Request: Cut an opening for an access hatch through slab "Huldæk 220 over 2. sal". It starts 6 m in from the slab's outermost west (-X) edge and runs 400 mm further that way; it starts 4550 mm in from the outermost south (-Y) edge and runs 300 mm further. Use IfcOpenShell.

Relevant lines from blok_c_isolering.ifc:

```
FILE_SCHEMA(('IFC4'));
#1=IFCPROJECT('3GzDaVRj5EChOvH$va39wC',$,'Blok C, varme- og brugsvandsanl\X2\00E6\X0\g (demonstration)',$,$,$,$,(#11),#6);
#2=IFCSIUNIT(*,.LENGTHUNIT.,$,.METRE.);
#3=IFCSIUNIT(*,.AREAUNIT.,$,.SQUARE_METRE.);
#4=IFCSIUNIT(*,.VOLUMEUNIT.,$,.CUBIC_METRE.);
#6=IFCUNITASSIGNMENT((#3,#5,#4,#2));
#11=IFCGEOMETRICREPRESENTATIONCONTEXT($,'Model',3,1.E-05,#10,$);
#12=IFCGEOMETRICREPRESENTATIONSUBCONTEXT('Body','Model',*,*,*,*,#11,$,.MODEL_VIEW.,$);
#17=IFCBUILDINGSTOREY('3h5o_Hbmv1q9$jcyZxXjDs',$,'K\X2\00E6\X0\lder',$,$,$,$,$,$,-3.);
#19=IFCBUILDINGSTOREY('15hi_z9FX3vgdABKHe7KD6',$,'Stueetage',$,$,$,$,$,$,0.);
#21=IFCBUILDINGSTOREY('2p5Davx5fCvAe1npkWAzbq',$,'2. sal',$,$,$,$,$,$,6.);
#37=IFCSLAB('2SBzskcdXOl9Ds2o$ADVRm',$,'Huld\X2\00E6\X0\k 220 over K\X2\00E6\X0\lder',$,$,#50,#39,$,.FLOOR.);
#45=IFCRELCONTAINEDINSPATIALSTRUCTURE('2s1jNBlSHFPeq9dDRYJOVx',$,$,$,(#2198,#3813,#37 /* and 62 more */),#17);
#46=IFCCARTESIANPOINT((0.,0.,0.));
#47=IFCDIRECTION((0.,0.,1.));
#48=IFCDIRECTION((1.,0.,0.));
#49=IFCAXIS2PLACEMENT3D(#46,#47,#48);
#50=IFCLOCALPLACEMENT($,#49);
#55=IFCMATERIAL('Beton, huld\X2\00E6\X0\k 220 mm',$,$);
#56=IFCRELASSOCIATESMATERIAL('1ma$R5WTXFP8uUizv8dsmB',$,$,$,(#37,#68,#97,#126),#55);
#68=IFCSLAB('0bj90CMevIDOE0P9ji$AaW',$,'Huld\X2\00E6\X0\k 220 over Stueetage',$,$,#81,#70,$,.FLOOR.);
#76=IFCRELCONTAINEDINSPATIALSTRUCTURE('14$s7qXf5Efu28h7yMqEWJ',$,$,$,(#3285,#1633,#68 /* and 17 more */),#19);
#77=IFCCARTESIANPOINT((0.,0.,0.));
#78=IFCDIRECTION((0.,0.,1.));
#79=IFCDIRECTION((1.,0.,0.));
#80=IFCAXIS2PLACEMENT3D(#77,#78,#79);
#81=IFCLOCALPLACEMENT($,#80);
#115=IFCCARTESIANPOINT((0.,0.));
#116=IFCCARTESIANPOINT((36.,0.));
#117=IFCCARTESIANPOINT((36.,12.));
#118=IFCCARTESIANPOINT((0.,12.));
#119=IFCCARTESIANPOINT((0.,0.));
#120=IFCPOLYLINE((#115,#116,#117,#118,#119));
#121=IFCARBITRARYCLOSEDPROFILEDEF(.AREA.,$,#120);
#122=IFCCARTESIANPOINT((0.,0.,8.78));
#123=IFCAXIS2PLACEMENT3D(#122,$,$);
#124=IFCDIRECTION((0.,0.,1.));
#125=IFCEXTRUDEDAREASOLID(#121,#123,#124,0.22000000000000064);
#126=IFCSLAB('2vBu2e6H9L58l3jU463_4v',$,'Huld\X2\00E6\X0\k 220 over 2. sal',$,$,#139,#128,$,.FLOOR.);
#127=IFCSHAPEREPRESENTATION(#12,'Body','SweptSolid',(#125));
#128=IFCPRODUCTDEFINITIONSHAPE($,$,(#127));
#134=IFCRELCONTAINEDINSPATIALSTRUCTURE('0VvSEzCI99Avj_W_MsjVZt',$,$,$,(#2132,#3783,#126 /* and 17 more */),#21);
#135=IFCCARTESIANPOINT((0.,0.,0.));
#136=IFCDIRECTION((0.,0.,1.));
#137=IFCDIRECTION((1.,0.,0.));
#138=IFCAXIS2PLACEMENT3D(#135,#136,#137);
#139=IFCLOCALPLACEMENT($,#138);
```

```python
import numpy as np
import ifcopenshell
import ifcopenshell.api.feature
import ifcopenshell.api.geometry
import ifcopenshell.api.root
import ifcopenshell.geom
import ifcopenshell.util.placement
import ifcopenshell.util.representation
import ifcopenshell.util.shape
import ifcopenshell.util.unit

model = ifcopenshell.open("blok_c_isolering.ifc")
unit_scale = ifcopenshell.util.unit.calculate_unit_scale(model)
settings = ifcopenshell.geom.settings()


def volume(element):
    """Net volume in cubic metres, openings subtracted."""
    shape = ifcopenshell.geom.create_shape(settings, element)
    return ifcopenshell.util.shape.get_volume(shape.geometry)


slab = model.by_id(126)
before = volume(slab)

# Extent in the slab's own axes, in metres. The edges named are its -X and -Y sides.
slab_shape = ifcopenshell.geom.create_shape(settings, slab)
vertices = ifcopenshell.util.shape.get_vertices(slab_shape.geometry)
x_min, y_min, bottom = vertices.min(axis=0)
top = vertices[:, 2].max()

opening = ifcopenshell.api.root.create_entity(model, ifc_class="IfcOpeningElement", name="Access hatch opening", predefined_type="OPENING")
context = ifcopenshell.util.representation.get_context(model, "Model", "Body", "MODEL_VIEW")
width, depth = 0.4, 0.3
outline = [(0.0, 0.0), (width, 0.0), (width, depth), (0.0, depth), (0.0, 0.0)]
# Overshoot both faces by 50 mm so the cut is clean.
shape = ifcopenshell.api.geometry.add_slab_representation(
    model, context=context, depth=top - bottom + 0.1, polyline=outline
)
ifcopenshell.api.geometry.assign_representation(model, product=opening, representation=shape)

matrix = ifcopenshell.util.placement.get_local_placement(slab.ObjectPlacement)
matrix[:, 3] = matrix @ np.append(np.array([x_min + 6, y_min + 4.55, bottom - 0.05]) / unit_scale, 1.0)
ifcopenshell.api.geometry.edit_object_placement(model, product=opening, matrix=matrix, is_si=False)
ifcopenshell.api.feature.add_feature(model, feature=opening, element=slab)

after = volume(slab)

print(f"slab volume {before:.3f} -> {after:.3f} m3")

model.write("blok_c_isolering_v2.ifc")
```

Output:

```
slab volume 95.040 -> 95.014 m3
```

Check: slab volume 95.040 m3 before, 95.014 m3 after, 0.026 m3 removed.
